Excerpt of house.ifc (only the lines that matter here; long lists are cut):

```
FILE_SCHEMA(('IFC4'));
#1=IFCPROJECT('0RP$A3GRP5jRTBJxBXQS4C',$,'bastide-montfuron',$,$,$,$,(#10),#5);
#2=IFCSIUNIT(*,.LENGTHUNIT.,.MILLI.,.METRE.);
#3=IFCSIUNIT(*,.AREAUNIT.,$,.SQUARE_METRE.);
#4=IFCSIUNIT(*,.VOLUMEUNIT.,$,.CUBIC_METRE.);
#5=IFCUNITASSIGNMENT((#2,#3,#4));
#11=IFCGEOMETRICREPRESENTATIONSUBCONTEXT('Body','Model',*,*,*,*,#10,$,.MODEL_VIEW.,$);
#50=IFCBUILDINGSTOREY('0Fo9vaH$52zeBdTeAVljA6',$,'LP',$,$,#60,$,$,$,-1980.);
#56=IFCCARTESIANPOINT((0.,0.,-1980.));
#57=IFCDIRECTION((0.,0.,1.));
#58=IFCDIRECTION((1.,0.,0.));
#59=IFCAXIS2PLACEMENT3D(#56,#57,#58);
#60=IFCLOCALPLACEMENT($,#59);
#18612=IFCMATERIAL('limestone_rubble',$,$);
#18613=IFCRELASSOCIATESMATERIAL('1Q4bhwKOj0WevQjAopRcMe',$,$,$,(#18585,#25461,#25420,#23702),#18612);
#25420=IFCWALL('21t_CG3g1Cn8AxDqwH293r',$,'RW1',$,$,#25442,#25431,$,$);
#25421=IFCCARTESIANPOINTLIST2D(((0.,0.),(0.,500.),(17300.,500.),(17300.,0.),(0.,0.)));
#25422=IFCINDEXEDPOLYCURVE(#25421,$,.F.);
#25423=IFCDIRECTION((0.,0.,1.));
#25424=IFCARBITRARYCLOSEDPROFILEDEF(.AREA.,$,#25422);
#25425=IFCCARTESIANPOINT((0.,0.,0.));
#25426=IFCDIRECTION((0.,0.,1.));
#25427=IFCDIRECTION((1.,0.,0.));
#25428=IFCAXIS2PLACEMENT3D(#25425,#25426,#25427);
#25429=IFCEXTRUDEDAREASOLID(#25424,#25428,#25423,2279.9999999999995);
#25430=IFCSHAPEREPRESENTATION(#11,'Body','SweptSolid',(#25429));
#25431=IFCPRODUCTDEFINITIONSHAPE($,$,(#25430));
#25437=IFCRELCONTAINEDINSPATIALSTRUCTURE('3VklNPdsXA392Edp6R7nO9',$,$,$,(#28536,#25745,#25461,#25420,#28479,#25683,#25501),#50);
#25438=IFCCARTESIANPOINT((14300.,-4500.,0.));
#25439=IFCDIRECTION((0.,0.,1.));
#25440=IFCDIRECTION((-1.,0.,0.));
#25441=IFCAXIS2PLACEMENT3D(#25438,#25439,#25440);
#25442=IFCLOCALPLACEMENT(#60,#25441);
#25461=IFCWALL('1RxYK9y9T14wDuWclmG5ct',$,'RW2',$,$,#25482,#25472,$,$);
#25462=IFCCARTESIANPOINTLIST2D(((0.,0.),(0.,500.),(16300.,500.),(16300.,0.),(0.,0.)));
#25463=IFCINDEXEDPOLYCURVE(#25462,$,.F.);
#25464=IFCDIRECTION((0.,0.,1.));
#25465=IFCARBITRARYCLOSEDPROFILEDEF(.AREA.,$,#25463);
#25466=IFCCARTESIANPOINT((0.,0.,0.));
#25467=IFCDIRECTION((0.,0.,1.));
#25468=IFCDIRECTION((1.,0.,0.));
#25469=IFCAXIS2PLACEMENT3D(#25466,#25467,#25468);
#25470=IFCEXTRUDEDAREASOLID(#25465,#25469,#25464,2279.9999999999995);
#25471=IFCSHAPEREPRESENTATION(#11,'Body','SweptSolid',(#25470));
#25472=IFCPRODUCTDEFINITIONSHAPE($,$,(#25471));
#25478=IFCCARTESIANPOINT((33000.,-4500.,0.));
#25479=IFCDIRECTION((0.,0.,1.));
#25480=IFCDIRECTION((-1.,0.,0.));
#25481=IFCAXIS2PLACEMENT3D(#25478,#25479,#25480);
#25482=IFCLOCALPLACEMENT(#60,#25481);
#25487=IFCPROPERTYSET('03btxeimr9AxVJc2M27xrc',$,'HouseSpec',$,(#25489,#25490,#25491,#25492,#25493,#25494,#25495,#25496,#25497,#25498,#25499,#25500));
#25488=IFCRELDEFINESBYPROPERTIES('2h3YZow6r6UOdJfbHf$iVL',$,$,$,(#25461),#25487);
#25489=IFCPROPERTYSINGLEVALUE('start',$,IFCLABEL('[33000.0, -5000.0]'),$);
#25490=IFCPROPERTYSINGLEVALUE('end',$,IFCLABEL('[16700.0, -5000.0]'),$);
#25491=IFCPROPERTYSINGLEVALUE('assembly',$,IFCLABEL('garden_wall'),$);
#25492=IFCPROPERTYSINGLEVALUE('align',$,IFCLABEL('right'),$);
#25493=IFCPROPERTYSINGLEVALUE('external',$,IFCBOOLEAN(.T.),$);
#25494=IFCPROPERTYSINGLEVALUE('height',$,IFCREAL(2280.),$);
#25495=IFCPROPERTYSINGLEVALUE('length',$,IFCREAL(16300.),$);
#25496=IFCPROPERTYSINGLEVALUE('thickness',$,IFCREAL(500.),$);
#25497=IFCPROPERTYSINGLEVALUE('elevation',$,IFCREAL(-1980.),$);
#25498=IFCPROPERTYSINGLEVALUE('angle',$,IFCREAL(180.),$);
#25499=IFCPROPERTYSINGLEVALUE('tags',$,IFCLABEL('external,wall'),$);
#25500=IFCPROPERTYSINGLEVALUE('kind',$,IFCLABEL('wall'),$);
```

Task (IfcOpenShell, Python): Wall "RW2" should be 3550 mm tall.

```python
import ifcopenshell
import ifcopenshell.api.pset
import ifcopenshell.geom
import ifcopenshell.util.element
import ifcopenshell.util.representation
import ifcopenshell.util.shape
import ifcopenshell.util.unit

model = ifcopenshell.open("house.ifc")
unit_scale = ifcopenshell.util.unit.calculate_unit_scale(model)
settings = ifcopenshell.geom.settings()


def volume(element):
    """Net volume in cubic metres, openings subtracted."""
    shape = ifcopenshell.geom.create_shape(settings, element)
    return ifcopenshell.util.shape.get_volume(shape.geometry)


wall = model.by_guid("1RxYK9y9T14wDuWclmG5ct")
before = volume(wall)

body = ifcopenshell.util.representation.get_representation(wall, "Model", "Body")
solid = body.Items[0]
old_height = solid.Depth
solid.Depth = 3.55 / unit_scale
after = volume(wall)

# Update the stored height, areas and volumes.
pset = model.by_id(ifcopenshell.util.element.get_pset(wall, "HouseSpec", should_inherit=False)["id"])
ifcopenshell.api.pset.edit_pset(model, pset=pset, properties={"height": model.create_entity("IfcReal", solid.Depth)})

print(f"height {old_height:g} -> {solid.Depth:g}, volume {before:.3f} -> {after:.3f} m3")

model.write("house_updated.ifc")
```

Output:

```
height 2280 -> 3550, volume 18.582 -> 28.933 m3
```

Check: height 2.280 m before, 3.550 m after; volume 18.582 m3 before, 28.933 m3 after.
